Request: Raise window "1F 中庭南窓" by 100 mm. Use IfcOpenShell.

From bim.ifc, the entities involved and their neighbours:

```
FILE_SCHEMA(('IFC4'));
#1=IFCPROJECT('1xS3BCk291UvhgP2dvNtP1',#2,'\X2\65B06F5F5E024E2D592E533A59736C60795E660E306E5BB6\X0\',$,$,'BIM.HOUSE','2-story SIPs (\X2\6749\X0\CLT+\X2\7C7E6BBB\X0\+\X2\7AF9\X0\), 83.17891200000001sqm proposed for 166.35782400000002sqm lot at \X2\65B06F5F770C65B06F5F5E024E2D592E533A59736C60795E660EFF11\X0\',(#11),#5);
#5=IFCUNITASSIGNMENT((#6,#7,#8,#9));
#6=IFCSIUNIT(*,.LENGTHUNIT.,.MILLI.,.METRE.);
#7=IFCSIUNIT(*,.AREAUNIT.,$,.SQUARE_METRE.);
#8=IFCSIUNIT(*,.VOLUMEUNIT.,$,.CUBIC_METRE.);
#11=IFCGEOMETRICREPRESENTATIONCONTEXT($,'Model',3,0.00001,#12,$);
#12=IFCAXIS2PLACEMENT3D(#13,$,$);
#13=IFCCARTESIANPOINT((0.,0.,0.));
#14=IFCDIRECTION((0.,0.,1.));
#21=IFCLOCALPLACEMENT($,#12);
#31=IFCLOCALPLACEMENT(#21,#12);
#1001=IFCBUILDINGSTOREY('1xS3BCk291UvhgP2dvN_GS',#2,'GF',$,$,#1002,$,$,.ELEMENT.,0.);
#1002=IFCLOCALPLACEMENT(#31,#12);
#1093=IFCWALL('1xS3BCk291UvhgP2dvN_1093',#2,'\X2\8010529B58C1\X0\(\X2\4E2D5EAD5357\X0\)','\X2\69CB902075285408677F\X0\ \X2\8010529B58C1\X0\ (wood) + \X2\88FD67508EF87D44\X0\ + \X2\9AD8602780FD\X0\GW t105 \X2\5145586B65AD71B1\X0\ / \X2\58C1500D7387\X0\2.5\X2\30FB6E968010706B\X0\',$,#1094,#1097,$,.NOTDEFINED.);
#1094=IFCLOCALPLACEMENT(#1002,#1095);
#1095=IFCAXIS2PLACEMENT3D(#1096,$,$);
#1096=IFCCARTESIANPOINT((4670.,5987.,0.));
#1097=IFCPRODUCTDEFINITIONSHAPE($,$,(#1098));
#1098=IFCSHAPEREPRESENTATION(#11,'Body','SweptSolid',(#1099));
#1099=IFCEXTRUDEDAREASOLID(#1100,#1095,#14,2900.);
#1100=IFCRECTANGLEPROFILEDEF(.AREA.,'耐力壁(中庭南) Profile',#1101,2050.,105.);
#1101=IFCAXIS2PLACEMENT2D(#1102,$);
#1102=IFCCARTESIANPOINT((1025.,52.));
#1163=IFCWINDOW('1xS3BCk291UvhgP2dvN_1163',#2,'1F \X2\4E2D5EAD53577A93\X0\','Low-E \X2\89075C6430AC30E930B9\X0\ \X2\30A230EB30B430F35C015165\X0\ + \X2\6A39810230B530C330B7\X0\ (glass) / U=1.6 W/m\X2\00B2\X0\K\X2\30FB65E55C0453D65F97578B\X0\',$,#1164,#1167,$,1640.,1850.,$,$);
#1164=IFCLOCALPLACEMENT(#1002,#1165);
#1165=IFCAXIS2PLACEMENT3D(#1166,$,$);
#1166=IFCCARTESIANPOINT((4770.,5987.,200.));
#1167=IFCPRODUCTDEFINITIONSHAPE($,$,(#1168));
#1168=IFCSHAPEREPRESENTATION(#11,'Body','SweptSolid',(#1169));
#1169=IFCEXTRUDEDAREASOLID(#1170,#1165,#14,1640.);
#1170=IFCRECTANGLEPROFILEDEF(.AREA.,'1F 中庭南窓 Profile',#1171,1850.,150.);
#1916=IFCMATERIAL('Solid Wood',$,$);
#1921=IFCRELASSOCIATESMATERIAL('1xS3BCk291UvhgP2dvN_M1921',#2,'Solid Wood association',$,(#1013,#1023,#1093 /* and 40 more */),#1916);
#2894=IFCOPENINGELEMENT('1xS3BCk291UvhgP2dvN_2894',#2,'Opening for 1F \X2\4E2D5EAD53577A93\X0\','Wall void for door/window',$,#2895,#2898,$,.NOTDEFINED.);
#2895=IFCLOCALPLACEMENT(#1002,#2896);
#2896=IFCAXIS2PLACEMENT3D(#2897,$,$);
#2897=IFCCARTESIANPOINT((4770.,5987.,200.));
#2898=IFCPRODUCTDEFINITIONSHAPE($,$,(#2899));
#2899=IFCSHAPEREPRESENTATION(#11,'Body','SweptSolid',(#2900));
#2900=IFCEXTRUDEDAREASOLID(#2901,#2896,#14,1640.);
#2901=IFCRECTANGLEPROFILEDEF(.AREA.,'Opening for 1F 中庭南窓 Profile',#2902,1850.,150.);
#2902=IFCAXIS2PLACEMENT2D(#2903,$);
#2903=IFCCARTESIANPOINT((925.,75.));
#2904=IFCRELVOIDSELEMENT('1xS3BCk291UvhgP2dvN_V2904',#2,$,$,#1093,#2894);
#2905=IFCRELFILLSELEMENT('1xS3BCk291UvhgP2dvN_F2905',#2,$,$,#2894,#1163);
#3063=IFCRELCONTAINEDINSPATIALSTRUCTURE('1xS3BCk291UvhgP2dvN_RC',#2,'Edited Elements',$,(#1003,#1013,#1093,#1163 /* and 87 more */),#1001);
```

```python
import numpy as np
import ifcopenshell
import ifcopenshell.api.geometry
import ifcopenshell.util.placement
import ifcopenshell.util.unit

model = ifcopenshell.open("bim.ifc")
unit_scale = ifcopenshell.util.unit.calculate_unit_scale(model)

window = model.by_id(1163)
opening = window.FillsVoids[0].RelatingOpeningElement
dz = 0.1 / unit_scale

shift = np.array([0.0, 0.0, dz])
# The window is not placed relative to its opening, so move both.
for product in (opening, window):
    matrix = ifcopenshell.util.placement.get_local_placement(product.ObjectPlacement)
    matrix[:3, 3] += shift
    ifcopenshell.api.geometry.edit_object_placement(model, product=product, matrix=matrix, is_si=False)

print(f"moved by {dz * unit_scale:+.3f} m")

model.write("bim_updated.ifc")
```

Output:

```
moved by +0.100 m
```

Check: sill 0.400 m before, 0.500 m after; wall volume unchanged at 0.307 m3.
